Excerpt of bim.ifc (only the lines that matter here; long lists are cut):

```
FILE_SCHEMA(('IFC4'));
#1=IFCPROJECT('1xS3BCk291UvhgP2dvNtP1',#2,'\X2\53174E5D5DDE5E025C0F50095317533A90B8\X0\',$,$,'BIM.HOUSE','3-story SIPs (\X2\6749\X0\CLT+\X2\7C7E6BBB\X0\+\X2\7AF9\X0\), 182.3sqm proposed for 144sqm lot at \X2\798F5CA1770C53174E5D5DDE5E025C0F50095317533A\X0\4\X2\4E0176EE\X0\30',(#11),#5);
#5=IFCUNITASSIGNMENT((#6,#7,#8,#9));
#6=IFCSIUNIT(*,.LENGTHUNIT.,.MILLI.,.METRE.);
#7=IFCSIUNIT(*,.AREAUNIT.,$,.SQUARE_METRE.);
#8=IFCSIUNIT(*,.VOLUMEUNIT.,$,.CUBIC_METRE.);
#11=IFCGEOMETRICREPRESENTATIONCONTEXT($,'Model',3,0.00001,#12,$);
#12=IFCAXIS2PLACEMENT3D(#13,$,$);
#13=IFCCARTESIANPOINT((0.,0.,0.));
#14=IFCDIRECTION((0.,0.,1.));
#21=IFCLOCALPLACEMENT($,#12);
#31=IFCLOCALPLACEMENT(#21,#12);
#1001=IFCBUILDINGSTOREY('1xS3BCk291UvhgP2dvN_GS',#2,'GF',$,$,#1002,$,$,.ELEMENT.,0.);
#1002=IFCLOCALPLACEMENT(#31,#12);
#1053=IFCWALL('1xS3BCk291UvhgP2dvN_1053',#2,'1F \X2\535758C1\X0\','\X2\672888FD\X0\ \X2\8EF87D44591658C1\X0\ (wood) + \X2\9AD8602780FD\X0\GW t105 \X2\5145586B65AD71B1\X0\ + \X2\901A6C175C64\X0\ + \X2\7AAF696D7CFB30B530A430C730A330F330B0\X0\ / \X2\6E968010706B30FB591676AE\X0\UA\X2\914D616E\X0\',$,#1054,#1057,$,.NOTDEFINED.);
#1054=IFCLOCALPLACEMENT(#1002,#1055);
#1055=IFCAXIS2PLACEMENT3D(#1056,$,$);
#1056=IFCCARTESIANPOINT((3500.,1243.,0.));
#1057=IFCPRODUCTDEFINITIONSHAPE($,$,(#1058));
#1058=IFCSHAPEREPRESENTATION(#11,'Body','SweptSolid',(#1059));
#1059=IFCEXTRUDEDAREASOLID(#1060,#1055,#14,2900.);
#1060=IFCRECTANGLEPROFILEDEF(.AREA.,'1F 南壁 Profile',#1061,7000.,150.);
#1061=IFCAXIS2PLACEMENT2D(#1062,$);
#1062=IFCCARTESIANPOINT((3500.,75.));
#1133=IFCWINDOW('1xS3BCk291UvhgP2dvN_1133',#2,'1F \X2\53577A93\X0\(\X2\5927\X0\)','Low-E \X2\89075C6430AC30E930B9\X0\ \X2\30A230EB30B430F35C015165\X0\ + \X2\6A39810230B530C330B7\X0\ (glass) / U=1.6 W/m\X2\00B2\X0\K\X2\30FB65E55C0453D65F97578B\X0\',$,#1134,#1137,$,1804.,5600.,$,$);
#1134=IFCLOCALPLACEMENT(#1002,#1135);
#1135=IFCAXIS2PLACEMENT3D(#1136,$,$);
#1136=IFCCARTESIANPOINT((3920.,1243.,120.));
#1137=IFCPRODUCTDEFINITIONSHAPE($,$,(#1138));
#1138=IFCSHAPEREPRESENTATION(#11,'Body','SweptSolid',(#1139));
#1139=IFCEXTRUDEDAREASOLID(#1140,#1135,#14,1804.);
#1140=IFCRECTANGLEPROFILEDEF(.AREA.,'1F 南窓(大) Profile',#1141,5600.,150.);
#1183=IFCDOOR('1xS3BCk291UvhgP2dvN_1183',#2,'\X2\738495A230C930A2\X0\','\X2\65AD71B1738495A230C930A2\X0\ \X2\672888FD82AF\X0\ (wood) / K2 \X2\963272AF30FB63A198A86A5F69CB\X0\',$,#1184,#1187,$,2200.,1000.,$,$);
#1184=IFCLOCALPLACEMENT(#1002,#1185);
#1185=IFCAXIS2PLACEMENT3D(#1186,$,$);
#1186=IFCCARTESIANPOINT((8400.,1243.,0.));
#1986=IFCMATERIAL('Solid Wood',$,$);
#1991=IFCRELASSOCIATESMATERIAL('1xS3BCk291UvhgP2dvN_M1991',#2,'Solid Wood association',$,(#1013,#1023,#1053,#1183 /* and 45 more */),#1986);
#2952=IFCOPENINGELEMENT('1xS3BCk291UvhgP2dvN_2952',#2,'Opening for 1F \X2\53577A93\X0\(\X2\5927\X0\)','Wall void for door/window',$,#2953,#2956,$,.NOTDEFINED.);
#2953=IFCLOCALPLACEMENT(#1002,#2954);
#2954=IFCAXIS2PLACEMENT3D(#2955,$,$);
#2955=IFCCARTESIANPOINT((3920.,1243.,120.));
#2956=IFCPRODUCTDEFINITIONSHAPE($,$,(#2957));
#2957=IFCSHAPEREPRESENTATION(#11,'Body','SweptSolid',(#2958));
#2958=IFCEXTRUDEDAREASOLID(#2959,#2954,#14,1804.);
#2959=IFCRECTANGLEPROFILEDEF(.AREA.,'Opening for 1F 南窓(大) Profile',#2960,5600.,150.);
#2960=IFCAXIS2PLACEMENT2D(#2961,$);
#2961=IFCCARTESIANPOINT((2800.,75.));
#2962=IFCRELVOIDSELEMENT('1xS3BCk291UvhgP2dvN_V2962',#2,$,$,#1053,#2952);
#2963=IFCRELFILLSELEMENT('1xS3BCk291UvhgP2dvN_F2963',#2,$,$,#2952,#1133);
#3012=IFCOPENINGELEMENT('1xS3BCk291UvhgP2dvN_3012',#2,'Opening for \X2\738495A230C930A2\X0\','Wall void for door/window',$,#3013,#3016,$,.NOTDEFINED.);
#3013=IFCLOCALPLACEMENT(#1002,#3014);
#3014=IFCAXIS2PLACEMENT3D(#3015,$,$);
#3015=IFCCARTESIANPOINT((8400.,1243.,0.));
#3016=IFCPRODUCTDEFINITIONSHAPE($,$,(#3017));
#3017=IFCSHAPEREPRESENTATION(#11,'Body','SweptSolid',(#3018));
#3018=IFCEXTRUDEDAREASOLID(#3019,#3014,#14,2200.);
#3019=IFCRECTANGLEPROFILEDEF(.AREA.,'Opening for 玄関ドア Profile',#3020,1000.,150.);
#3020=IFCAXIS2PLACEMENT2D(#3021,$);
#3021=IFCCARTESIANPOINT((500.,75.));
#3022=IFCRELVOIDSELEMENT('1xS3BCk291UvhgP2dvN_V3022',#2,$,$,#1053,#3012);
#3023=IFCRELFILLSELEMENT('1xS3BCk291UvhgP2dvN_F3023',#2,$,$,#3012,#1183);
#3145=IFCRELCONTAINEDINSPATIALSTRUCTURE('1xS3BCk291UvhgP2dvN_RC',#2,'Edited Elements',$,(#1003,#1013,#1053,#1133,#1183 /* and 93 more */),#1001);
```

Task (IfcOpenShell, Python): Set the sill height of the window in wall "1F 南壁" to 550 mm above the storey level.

```python
import numpy as np
import ifcopenshell
import ifcopenshell.api.geometry
import ifcopenshell.geom
import ifcopenshell.util.element
import ifcopenshell.util.placement
import ifcopenshell.util.shape
import ifcopenshell.util.unit

model = ifcopenshell.open("bim.ifc")
unit_scale = ifcopenshell.util.unit.calculate_unit_scale(model)

window = model.by_guid("1xS3BCk291UvhgP2dvN_1133")
opening = window.FillsVoids[0].RelatingOpeningElement
storey = ifcopenshell.util.element.get_container(window, ifc_class="IfcBuildingStorey")
level = ifcopenshell.util.placement.get_local_placement(storey.ObjectPlacement)[2, 3]

# The opening's origin need not be at the sill, so measure its lowest point.
shape = ifcopenshell.geom.create_shape(ifcopenshell.geom.settings(), opening)
bottom = ifcopenshell.util.shape.get_shape_bottom_elevation(shape, shape.geometry) / unit_scale
dz = level + 0.55 / unit_scale - bottom

shift = np.array([0.0, 0.0, dz])
# The window is not placed relative to its opening, so move both.
for product in (opening, window):
    matrix = ifcopenshell.util.placement.get_local_placement(product.ObjectPlacement)
    matrix[:3, 3] += shift
    ifcopenshell.api.geometry.edit_object_placement(model, product=product, matrix=matrix, is_si=False)

print(f"moved by {dz * unit_scale:+.3f} m")

model.write("bim_edited.ifc")
```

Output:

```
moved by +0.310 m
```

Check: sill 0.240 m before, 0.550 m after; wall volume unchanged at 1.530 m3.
